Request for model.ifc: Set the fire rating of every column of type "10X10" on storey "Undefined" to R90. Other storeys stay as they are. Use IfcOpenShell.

First a look at what the model holds.

```python
import ifcopenshell
import ifcopenshell.util.element

model = ifcopenshell.open("model.ifc")
print(model.schema)
storey = next(s for s in model.by_type("IfcBuildingStorey") if s.Name == "Undefined")
columns = [e for e in ifcopenshell.util.element.get_decomposition(storey) if e.is_a("IfcColumn")]
seen = {}
for e in columns:
    element_type = ifcopenshell.util.element.get_type(e)
    key = (element_type.Name if element_type != e and element_type else None, ifcopenshell.util.element.get_pset(e, "Pset_ColumnCommon", "FireRating"))
    seen[key] = seen.get(key, 0) + 1
for (name, value), count in sorted(seen.items(), key=str):
    print(count, "x", name, "|", value)
```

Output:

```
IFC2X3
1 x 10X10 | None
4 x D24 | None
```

```python
import ifcopenshell
import ifcopenshell.api.pset
import ifcopenshell.util.element

model = ifcopenshell.open("model.ifc")

storey = next(s for s in model.by_type("IfcBuildingStorey") if s.Name == "Undefined")
columns = [e for e in ifcopenshell.util.element.get_decomposition(storey) if e.is_a("IfcColumn")]

count = 0
for e in columns:
    element_type = ifcopenshell.util.element.get_type(e)
    if element_type in (None, e) or element_type.Name != "10X10":
        continue
    # add_pset returns the element's existing set when there is one.
    pset = ifcopenshell.api.pset.add_pset(model, product=e, name="Pset_ColumnCommon")
    ifcopenshell.api.pset.edit_pset(model, pset=pset, properties={"FireRating": "R90"})
    count += 1

print(count, "columns updated")

model.write("model_v2.ifc")
```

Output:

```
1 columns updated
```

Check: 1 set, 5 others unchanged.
